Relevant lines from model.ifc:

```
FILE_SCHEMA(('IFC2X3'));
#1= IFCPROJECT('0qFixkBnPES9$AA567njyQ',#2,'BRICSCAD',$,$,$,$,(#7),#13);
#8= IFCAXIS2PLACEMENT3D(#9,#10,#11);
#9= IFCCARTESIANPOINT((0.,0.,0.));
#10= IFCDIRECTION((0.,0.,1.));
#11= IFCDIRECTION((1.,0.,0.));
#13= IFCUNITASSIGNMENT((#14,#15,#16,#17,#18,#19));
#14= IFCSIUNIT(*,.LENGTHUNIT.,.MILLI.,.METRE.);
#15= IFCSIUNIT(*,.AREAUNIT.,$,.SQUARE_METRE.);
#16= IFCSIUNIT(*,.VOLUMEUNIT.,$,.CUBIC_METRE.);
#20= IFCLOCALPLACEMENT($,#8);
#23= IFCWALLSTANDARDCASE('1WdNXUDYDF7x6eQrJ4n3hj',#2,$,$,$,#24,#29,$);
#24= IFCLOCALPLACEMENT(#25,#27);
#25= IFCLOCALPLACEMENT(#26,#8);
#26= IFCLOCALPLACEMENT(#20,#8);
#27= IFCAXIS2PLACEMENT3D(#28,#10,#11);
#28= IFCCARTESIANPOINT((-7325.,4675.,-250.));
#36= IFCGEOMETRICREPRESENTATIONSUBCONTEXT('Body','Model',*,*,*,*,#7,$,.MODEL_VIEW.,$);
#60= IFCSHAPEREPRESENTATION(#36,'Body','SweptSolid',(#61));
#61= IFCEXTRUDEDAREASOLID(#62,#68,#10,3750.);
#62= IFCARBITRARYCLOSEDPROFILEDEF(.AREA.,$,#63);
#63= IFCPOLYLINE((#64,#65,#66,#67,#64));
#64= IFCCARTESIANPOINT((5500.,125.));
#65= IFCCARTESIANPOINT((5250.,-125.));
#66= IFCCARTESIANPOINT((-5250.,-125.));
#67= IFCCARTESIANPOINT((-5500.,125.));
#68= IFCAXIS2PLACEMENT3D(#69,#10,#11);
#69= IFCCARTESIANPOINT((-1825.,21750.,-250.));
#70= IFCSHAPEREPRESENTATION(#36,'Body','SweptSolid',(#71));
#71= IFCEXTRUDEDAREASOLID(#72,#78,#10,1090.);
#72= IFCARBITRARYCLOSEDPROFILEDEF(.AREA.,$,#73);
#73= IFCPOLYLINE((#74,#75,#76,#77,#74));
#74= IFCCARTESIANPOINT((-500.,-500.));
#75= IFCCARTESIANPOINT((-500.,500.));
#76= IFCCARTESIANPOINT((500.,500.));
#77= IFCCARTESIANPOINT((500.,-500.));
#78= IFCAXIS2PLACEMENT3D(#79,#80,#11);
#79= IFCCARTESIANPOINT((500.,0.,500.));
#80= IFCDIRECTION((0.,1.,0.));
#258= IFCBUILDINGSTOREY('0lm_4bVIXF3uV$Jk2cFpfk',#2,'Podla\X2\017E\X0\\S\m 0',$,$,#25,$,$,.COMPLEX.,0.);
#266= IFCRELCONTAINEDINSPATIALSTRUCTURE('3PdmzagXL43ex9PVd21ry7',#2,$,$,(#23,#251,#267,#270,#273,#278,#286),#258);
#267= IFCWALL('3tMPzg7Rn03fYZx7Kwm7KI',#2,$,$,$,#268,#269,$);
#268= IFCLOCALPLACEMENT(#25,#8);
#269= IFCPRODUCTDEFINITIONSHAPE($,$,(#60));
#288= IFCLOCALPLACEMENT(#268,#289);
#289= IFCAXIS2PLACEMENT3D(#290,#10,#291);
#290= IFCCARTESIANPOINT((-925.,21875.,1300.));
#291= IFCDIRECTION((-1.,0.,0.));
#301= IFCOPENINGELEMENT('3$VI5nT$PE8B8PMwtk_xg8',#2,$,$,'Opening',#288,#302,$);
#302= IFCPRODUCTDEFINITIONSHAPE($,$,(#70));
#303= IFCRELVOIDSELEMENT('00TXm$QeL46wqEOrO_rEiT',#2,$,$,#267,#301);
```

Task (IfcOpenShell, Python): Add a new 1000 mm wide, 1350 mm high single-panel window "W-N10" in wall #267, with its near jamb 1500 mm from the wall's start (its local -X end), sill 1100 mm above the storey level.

```python
import numpy as np
import ifcopenshell
import ifcopenshell.api.feature
import ifcopenshell.api.geometry
import ifcopenshell.api.root
import ifcopenshell.api.spatial
import ifcopenshell.api.type
import ifcopenshell.geom
import ifcopenshell.util.element
import ifcopenshell.util.placement
import ifcopenshell.util.representation
import ifcopenshell.util.shape
import ifcopenshell.util.unit

model = ifcopenshell.open("model.ifc")
unit_scale = ifcopenshell.util.unit.calculate_unit_scale(model)
settings = ifcopenshell.geom.settings()


def volume(element):
    """Net volume in cubic metres, openings subtracted."""
    shape = ifcopenshell.geom.create_shape(settings, element)
    return ifcopenshell.util.shape.get_volume(shape.geometry)


wall = model.by_guid("3tMPzg7Rn03fYZx7Kwm7KI")
storey = ifcopenshell.util.element.get_container(wall, ifc_class="IfcBuildingStorey")
context = ifcopenshell.util.representation.get_context(model, "Model", "Body", "MODEL_VIEW")
before = volume(wall)

width, height, from_end, sill = 1, 1.35, 1.5, 1.1  # metres

# The wall runs along its own X axis, and the end named is its -X end.
wall_shape = ifcopenshell.geom.create_shape(settings, wall)
x, y, z = ifcopenshell.util.shape.get_vertices(wall_shape.geometry).T
start = x.min() + from_end
face, thickness = float(y.min()), float(y.max() - y.min())
wall_matrix = ifcopenshell.util.placement.get_local_placement(wall.ObjectPlacement)
level = ifcopenshell.util.placement.get_local_placement(storey.ObjectPlacement)[2, 3]


def in_wall(x, y):
    """Placement at x, y metres in the wall's axes, at sill height."""
    matrix = wall_matrix.copy()
    matrix[:, 3] = wall_matrix @ np.array([x / unit_scale, y / unit_scale, 0.0, 1.0])
    matrix[2, 3] = level + sill / unit_scale
    return matrix


# Opening: a box that overshoots both wall faces by 50 mm.
opening = ifcopenshell.api.root.create_entity(model, ifc_class="IfcOpeningElement")
box = ifcopenshell.api.geometry.add_wall_representation(
    model, context=context, length=width, height=height, thickness=thickness + 0.1
)
ifcopenshell.api.geometry.assign_representation(model, product=opening, representation=box)
ifcopenshell.api.geometry.edit_object_placement(model, product=opening, matrix=in_wall(start, face - 0.05), is_si=False)
ifcopenshell.api.feature.add_feature(model, feature=opening, element=wall)

window = ifcopenshell.api.root.create_entity(model, ifc_class="IfcWindow", name="W-N10")
window.OverallWidth, window.OverallHeight = width / unit_scale, height / unit_scale
body = ifcopenshell.api.geometry.add_window_representation(
    model,
    context=context,
    overall_width=window.OverallWidth,
    overall_height=window.OverallHeight,
    partition_type="SINGLE_PANEL",
)
ifcopenshell.api.geometry.assign_representation(model, product=window, representation=body)
ifcopenshell.api.spatial.assign_container(model, products=[window], relating_structure=storey)
fills = ifcopenshell.api.feature.add_filling(model, opening=opening, element=window)
fills.OwnerHistory = window.OwnerHistory  # required in IFC2X3

# IFC2X3 keeps the operation on the window style.
style = ifcopenshell.api.root.create_entity(model, ifc_class="IfcWindowStyle", name="W-N10")
style.OperationType, style.ConstructionType = "SINGLE_PANEL", "NOTDEFINED"
style.ParameterTakesPrecedence = style.Sizeable = False
ifcopenshell.api.type.assign_type(model, related_objects=[window], relating_type=style)

# Centre the window in the wall's thickness.
ifcopenshell.api.geometry.edit_object_placement(model, product=window, matrix=in_wall(start, face), is_si=False)
window_shape = ifcopenshell.geom.create_shape(settings, window)
depth = ifcopenshell.util.shape.get_vertices(window_shape.geometry)[:, 1]
offset = face + thickness / 2 - (depth.min() + depth.max()) / 2
ifcopenshell.api.geometry.edit_object_placement(model, product=window, matrix=in_wall(start, offset), is_si=False)

after = volume(wall)

print(f"wall volume {before:.3f} -> {after:.3f} m3")

model.write("model_edited.ifc")
```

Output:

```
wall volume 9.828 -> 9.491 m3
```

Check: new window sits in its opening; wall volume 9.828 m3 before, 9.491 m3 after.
